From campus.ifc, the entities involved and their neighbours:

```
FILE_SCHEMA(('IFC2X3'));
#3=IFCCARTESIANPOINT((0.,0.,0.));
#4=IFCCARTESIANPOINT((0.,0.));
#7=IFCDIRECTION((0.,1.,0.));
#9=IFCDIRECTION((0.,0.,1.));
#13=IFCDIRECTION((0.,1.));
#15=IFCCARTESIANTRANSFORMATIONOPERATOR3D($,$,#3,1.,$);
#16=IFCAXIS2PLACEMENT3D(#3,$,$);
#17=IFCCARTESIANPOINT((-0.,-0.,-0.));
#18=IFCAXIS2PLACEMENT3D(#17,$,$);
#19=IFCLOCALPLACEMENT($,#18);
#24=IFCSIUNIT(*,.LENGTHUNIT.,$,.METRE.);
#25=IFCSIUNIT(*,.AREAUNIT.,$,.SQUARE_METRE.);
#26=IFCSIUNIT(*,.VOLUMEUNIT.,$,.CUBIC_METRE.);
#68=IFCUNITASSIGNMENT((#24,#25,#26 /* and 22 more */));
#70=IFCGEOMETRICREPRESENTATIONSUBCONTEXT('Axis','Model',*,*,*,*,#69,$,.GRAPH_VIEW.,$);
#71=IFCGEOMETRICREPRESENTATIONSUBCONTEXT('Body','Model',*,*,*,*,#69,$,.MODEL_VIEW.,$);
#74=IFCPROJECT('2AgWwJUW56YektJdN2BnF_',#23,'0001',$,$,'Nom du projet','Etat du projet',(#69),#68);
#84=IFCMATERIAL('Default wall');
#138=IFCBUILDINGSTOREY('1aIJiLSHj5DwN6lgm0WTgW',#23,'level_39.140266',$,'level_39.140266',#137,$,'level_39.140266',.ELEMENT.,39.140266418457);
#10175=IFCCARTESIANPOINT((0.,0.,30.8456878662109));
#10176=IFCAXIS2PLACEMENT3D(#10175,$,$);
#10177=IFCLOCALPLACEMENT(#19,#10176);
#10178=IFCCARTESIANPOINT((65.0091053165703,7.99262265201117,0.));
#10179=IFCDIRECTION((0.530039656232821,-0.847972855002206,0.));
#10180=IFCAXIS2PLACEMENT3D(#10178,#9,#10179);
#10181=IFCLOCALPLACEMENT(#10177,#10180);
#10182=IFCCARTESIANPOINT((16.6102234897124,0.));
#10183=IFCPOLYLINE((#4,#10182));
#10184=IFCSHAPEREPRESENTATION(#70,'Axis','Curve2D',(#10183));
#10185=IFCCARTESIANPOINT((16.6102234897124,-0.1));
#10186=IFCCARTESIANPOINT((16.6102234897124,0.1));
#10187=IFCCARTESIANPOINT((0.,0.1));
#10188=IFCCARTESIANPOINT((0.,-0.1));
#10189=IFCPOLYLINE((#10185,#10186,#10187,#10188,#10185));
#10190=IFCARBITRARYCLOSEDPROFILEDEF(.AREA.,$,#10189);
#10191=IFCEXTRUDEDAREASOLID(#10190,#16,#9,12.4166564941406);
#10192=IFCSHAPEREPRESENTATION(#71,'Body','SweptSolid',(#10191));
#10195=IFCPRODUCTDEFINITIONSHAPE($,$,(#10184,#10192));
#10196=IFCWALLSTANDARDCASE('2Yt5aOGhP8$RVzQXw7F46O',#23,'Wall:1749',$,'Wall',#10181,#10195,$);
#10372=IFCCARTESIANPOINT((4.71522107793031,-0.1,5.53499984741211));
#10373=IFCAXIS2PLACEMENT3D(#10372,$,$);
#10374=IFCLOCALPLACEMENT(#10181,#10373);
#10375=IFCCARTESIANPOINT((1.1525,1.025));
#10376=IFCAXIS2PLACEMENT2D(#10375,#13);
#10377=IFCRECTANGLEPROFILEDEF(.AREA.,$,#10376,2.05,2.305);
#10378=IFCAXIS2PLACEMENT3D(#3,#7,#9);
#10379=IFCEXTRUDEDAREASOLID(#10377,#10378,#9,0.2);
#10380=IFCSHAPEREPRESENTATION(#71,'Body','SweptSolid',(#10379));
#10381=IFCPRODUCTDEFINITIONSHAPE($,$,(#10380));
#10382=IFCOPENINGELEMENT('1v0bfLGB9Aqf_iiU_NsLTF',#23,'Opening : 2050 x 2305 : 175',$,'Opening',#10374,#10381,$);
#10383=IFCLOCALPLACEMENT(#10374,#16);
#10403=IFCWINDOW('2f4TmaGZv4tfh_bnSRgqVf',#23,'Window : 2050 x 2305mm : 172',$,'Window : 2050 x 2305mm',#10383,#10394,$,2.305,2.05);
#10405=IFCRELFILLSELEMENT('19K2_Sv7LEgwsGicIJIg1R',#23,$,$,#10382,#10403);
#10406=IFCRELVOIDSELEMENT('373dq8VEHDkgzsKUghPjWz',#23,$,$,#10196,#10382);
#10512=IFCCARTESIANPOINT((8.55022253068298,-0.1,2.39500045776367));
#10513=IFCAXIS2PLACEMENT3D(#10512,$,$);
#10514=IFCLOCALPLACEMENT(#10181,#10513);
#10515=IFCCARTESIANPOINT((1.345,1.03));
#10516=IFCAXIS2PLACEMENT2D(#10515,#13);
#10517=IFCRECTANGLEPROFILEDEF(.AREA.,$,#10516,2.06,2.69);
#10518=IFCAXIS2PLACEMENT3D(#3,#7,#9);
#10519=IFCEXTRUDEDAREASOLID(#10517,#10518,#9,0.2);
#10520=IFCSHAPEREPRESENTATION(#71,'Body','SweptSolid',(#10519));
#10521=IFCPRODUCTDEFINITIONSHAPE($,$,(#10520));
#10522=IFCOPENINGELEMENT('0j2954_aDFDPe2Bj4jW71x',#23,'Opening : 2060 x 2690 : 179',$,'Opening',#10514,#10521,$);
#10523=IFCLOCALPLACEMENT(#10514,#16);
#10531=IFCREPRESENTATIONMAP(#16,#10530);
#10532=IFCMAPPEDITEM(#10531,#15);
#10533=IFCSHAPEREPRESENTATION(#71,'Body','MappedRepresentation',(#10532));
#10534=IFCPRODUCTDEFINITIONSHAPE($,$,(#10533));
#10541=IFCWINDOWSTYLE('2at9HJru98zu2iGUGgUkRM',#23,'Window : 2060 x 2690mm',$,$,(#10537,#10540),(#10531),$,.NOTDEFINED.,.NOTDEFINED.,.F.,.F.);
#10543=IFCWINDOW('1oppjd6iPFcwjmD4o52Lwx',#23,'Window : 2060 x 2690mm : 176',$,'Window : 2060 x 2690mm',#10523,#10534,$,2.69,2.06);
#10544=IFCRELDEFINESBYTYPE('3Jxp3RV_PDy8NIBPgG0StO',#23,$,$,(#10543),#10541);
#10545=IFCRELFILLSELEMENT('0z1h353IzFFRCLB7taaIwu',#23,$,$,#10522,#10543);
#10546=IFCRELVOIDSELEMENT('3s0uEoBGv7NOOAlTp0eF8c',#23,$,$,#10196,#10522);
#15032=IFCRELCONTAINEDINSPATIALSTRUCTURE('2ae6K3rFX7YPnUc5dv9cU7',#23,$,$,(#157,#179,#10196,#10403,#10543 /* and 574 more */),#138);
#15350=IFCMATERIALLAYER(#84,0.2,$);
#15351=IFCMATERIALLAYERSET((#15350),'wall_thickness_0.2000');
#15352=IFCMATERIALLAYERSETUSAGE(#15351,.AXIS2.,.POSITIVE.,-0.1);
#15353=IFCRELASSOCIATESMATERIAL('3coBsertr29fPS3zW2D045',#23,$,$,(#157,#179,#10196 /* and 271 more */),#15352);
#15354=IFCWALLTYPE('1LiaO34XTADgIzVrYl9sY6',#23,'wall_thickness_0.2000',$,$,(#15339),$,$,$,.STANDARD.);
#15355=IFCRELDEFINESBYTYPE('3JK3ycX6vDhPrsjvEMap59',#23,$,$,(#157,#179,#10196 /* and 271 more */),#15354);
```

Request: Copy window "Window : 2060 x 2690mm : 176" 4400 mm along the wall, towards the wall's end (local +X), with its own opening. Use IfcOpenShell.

```python
import ifcopenshell
import ifcopenshell.api.feature
import ifcopenshell.api.geometry
import ifcopenshell.api.root
import ifcopenshell.geom
import ifcopenshell.util.element
import ifcopenshell.util.placement
import ifcopenshell.util.shape

model = ifcopenshell.open("campus.ifc")
settings = ifcopenshell.geom.settings()


def volume(element):
    """Net volume in cubic metres, openings subtracted."""
    shape = ifcopenshell.geom.create_shape(settings, element)
    return ifcopenshell.util.shape.get_volume(shape.geometry)


window = model.by_id(10543)
opening = window.FillsVoids[0].RelatingOpeningElement
wall = opening.VoidsElements[0].RelatingBuildingElement
before = volume(wall)
shift = ifcopenshell.util.placement.get_local_placement(wall.ObjectPlacement)[:3, 0] * 4.4

# copy_class copies the void relationship, type, container and properties, but no geometry.
new_opening = ifcopenshell.api.root.copy_class(model, product=opening)
new_opening.Representation = ifcopenshell.util.element.copy_deep(
    model, opening.Representation, exclude=["IfcGeometricRepresentationContext", "IfcRepresentationMap"]
)
new_opening.Name = "Opening : 2060 x 2690"
new_window = ifcopenshell.api.root.copy_class(model, product=window)
new_window.Representation = ifcopenshell.util.element.copy_deep(
    model, window.Representation, exclude=["IfcGeometricRepresentationContext", "IfcRepresentationMap"]
)
new_window.Name = "Window : 2060 x 2690mm"
fills = ifcopenshell.api.feature.add_filling(model, opening=new_opening, element=new_window)
fills.OwnerHistory = new_window.OwnerHistory  # required in IFC2X3

for old, new in ((opening, new_opening), (window, new_window)):
    matrix = ifcopenshell.util.placement.get_local_placement(old.ObjectPlacement)
    matrix[:3, 3] += shift
    ifcopenshell.api.geometry.edit_object_placement(model, product=new, matrix=matrix, is_si=False)

after = volume(wall)

print(f"wall volume {before:.3f} -> {after:.3f} m3")

model.write("campus-out.ifc")
```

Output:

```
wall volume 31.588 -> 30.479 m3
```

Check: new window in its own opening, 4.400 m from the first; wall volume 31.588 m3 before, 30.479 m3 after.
